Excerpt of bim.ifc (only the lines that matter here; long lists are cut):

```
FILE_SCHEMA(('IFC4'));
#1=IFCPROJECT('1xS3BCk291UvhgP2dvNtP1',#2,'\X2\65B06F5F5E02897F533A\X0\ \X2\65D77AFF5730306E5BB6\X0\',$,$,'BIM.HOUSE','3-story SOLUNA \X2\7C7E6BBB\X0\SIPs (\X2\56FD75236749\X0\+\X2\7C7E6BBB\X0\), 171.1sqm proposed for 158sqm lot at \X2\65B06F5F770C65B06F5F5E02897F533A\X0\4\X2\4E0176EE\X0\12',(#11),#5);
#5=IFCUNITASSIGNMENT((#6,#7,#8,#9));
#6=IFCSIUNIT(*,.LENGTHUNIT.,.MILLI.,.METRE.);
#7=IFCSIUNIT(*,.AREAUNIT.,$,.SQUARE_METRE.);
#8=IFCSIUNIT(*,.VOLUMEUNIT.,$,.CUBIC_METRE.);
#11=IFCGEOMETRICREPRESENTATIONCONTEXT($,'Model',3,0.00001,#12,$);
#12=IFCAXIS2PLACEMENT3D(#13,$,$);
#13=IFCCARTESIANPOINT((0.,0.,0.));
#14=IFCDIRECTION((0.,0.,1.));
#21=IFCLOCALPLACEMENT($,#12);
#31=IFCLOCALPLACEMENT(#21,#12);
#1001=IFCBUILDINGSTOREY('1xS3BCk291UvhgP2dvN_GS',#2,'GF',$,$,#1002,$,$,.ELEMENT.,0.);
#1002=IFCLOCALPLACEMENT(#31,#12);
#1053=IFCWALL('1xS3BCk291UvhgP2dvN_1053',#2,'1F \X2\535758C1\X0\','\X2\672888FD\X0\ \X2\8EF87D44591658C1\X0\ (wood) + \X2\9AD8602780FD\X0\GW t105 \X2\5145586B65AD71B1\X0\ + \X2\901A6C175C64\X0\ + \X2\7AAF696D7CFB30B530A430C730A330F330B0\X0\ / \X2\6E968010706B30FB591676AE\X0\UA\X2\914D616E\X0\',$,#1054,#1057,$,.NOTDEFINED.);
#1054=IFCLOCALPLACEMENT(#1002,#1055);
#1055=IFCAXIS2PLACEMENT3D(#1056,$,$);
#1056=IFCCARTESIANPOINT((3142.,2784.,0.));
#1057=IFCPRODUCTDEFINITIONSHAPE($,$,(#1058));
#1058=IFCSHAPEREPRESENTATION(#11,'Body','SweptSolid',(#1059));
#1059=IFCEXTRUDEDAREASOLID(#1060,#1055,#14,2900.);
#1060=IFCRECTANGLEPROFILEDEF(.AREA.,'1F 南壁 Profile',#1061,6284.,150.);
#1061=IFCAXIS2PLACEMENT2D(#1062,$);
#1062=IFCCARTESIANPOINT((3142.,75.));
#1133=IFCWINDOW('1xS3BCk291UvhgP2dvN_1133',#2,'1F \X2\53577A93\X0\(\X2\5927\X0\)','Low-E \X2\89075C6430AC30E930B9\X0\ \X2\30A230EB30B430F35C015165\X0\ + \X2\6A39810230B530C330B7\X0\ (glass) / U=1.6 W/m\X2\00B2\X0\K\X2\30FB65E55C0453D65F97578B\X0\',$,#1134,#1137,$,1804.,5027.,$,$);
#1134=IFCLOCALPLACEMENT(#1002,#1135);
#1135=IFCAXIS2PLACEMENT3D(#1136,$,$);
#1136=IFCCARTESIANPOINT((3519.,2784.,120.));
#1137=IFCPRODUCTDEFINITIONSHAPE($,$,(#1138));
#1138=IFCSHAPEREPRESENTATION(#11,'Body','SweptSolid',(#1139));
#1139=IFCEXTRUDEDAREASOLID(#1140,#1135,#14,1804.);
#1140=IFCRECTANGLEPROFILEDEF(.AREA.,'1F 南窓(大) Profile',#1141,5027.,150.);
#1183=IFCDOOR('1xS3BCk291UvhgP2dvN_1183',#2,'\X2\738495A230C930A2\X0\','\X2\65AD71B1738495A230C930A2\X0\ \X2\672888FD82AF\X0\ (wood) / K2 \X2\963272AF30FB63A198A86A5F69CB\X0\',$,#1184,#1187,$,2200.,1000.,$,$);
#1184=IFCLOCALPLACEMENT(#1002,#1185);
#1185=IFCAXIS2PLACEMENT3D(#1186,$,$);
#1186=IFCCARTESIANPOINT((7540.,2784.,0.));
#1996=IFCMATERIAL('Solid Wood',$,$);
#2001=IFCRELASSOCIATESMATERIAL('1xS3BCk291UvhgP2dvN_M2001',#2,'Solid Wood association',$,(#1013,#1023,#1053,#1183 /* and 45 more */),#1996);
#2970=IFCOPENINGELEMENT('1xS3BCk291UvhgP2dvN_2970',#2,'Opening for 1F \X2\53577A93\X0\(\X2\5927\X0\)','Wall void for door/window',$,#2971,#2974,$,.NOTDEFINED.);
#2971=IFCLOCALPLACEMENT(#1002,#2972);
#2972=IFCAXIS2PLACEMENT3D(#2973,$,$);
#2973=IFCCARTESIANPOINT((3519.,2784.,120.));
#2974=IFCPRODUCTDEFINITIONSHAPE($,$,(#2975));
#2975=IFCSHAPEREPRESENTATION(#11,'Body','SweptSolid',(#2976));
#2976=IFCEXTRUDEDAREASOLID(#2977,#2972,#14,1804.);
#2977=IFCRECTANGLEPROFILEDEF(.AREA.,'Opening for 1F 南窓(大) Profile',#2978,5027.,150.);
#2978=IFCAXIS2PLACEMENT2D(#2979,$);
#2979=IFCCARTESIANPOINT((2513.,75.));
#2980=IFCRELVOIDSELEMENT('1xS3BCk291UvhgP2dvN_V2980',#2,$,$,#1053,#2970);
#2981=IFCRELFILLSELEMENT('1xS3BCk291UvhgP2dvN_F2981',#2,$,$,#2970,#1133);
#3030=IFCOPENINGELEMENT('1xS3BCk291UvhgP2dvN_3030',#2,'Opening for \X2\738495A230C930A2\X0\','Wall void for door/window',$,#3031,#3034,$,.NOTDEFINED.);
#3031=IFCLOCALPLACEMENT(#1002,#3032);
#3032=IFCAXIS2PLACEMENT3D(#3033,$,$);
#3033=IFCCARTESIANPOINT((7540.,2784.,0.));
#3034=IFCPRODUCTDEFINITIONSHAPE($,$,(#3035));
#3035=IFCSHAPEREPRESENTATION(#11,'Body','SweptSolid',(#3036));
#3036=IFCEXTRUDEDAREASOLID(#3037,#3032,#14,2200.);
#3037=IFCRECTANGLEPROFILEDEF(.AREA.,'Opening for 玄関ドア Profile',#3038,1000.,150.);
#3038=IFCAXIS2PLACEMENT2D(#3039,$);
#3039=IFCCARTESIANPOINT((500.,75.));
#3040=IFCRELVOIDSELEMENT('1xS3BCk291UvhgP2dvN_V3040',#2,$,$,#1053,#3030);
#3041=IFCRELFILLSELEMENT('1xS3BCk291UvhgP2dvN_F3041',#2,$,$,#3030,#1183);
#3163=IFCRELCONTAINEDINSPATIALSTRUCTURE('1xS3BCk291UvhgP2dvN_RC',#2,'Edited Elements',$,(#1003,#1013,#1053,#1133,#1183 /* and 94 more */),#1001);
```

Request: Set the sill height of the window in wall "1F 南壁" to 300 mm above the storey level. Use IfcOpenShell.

```python
import numpy as np
import ifcopenshell
import ifcopenshell.api.geometry
import ifcopenshell.geom
import ifcopenshell.util.element
import ifcopenshell.util.placement
import ifcopenshell.util.shape
import ifcopenshell.util.unit

model = ifcopenshell.open("bim.ifc")
unit_scale = ifcopenshell.util.unit.calculate_unit_scale(model)

window = model.by_guid("1xS3BCk291UvhgP2dvN_1133")
opening = window.FillsVoids[0].RelatingOpeningElement
storey = ifcopenshell.util.element.get_container(window, ifc_class="IfcBuildingStorey")
level = ifcopenshell.util.placement.get_local_placement(storey.ObjectPlacement)[2, 3]

# The opening's origin need not be at the sill, so measure its lowest point.
shape = ifcopenshell.geom.create_shape(ifcopenshell.geom.settings(), opening)
bottom = ifcopenshell.util.shape.get_shape_bottom_elevation(shape, shape.geometry) / unit_scale
dz = level + 0.3 / unit_scale - bottom

shift = np.array([0.0, 0.0, dz])
# The window is not placed relative to its opening, so move both.
for product in (opening, window):
    matrix = ifcopenshell.util.placement.get_local_placement(product.ObjectPlacement)
    matrix[:3, 3] += shift
    ifcopenshell.api.geometry.edit_object_placement(model, product=product, matrix=matrix, is_si=False)

print(f"moved by {dz * unit_scale:+.3f} m")

model.write("bim-out.ifc")
```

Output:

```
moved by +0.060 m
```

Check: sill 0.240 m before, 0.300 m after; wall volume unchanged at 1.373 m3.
